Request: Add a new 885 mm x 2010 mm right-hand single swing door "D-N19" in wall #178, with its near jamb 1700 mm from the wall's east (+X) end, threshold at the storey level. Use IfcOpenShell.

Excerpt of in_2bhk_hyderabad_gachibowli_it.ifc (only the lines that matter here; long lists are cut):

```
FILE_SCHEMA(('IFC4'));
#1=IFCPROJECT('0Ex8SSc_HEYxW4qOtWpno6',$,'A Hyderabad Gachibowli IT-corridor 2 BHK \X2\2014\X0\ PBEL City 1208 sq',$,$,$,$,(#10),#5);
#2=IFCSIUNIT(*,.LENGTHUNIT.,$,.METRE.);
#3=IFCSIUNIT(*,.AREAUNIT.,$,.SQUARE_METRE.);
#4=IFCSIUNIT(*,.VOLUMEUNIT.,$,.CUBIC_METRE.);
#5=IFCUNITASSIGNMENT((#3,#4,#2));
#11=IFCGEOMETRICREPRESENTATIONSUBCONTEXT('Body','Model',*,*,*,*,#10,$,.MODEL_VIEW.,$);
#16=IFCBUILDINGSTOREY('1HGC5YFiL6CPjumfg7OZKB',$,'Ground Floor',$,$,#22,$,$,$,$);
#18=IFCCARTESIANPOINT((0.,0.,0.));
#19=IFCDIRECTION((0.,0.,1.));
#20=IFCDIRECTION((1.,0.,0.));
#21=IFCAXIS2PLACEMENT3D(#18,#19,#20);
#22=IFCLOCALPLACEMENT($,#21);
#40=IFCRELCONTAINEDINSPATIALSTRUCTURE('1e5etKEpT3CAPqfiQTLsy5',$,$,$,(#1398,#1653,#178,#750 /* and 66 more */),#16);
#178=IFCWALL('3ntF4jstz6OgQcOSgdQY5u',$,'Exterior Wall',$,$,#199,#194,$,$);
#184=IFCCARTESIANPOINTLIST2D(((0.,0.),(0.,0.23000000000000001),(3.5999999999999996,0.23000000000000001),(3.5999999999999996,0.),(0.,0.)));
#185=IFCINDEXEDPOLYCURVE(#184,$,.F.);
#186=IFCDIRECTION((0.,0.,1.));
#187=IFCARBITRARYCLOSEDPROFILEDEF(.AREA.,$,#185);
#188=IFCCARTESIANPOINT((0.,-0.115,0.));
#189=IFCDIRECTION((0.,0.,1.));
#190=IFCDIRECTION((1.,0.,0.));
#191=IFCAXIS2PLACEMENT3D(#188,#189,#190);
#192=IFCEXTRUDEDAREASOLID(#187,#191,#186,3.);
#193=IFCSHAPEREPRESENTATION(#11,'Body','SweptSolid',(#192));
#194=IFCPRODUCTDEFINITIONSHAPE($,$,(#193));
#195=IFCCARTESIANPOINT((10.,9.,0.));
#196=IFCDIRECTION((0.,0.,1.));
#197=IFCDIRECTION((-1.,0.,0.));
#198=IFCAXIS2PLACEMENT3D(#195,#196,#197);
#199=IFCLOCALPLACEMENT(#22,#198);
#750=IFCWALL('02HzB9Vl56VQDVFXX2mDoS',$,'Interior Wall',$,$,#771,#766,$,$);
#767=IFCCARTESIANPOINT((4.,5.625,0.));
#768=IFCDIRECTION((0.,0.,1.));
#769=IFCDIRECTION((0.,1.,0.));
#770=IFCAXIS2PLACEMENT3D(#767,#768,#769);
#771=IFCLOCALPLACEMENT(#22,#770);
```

```python
import numpy as np
import ifcopenshell
import ifcopenshell.api.feature
import ifcopenshell.api.geometry
import ifcopenshell.api.root
import ifcopenshell.api.spatial
import ifcopenshell.geom
import ifcopenshell.util.element
import ifcopenshell.util.placement
import ifcopenshell.util.representation
import ifcopenshell.util.shape
import ifcopenshell.util.unit

model = ifcopenshell.open("in_2bhk_hyderabad_gachibowli_it.ifc")
unit_scale = ifcopenshell.util.unit.calculate_unit_scale(model)
settings = ifcopenshell.geom.settings()


def volume(element):
    """Net volume in cubic metres, openings subtracted."""
    shape = ifcopenshell.geom.create_shape(settings, element)
    return ifcopenshell.util.shape.get_volume(shape.geometry)


wall = model.by_guid("3ntF4jstz6OgQcOSgdQY5u")
storey = ifcopenshell.util.element.get_container(wall, ifc_class="IfcBuildingStorey")
context = ifcopenshell.util.representation.get_context(model, "Model", "Body", "MODEL_VIEW")
before = volume(wall)

width, height, from_end, sill = 0.885, 2.01, 1.7, 0.0  # metres

# The wall runs along its own X axis, and the end named is its -X end.
wall_shape = ifcopenshell.geom.create_shape(settings, wall)
x, y, z = ifcopenshell.util.shape.get_vertices(wall_shape.geometry).T
start = x.min() + from_end
face, thickness = float(y.min()), float(y.max() - y.min())
wall_matrix = ifcopenshell.util.placement.get_local_placement(wall.ObjectPlacement)
level = ifcopenshell.util.placement.get_local_placement(storey.ObjectPlacement)[2, 3]


def in_wall(x, y):
    """Placement at x, y metres in the wall's axes, at sill height."""
    matrix = wall_matrix.copy()
    matrix[:, 3] = wall_matrix @ np.array([x / unit_scale, y / unit_scale, 0.0, 1.0])
    matrix[2, 3] = level + sill / unit_scale
    return matrix


# Opening: a box that overshoots both wall faces by 50 mm.
opening = ifcopenshell.api.root.create_entity(model, ifc_class="IfcOpeningElement", predefined_type="OPENING")
box = ifcopenshell.api.geometry.add_wall_representation(
    model, context=context, length=width, height=height, thickness=thickness + 0.1
)
ifcopenshell.api.geometry.assign_representation(model, product=opening, representation=box)
ifcopenshell.api.geometry.edit_object_placement(model, product=opening, matrix=in_wall(start, face - 0.05), is_si=False)
ifcopenshell.api.feature.add_feature(model, feature=opening, element=wall)

door = ifcopenshell.api.root.create_entity(model, ifc_class="IfcDoor", name="D-N19", predefined_type="DOOR")
door.OverallWidth, door.OverallHeight = width / unit_scale, height / unit_scale
door.OperationType = "SINGLE_SWING_RIGHT"
body = ifcopenshell.api.geometry.add_door_representation(
    model,
    context=context,
    overall_width=door.OverallWidth,
    overall_height=door.OverallHeight,
    operation_type="SINGLE_SWING_RIGHT",
    lining_properties={"LiningDepth": thickness / unit_scale, "ThresholdDepth": thickness / unit_scale},
)
ifcopenshell.api.geometry.assign_representation(model, product=door, representation=body)
ifcopenshell.api.spatial.assign_container(model, products=[door], relating_structure=storey)
ifcopenshell.api.feature.add_filling(model, opening=opening, element=door)

# The lining spans the wall, so the door starts at the wall face.
ifcopenshell.api.geometry.edit_object_placement(model, product=door, matrix=in_wall(start, face), is_si=False)

after = volume(wall)

print(f"wall volume {before:.3f} -> {after:.3f} m3")

model.write("in_2bhk_hyderabad_gachibowli_it_updated.ifc")
```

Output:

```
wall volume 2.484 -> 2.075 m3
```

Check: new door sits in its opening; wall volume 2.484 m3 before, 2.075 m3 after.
